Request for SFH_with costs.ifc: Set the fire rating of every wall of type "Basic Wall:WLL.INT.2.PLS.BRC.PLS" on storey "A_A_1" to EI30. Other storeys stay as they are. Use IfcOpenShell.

First a look at what the model holds.

```python
import ifcopenshell
import ifcopenshell.util.element

model = ifcopenshell.open("SFH_with costs.ifc")
print(model.schema)
storey = next(s for s in model.by_type("IfcBuildingStorey") if s.Name == "A_A_1")
walls = [e for e in ifcopenshell.util.element.get_decomposition(storey) if e.is_a("IfcWall")]
seen = {}
for e in walls:
    element_type = ifcopenshell.util.element.get_type(e)
    key = (element_type.Name if element_type != e and element_type else None, ifcopenshell.util.element.get_pset(e, "Pset_WallCommon", "FireRating"))
    seen[key] = seen.get(key, 0) + 1
for (name, value), count in sorted(seen.items(), key=str):
    print(count, "x", name, "|", value)
```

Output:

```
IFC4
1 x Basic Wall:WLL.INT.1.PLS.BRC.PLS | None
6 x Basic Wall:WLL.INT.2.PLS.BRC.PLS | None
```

```python
import ifcopenshell
import ifcopenshell.api.pset
import ifcopenshell.util.element

model = ifcopenshell.open("SFH_with costs.ifc")

storey = next(s for s in model.by_type("IfcBuildingStorey") if s.Name == "A_A_1")
walls = [e for e in ifcopenshell.util.element.get_decomposition(storey) if e.is_a("IfcWall")]

count = 0
for e in walls:
    element_type = ifcopenshell.util.element.get_type(e)
    if element_type in (None, e) or element_type.Name != "Basic Wall:WLL.INT.2.PLS.BRC.PLS":
        continue
    # add_pset returns the element's existing set when there is one.
    pset = ifcopenshell.api.pset.add_pset(model, product=e, name="Pset_WallCommon")
    ifcopenshell.api.pset.edit_pset(model, pset=pset, properties={"FireRating": "EI30"})
    count += 1

print(count, "walls updated")

model.write("SFH_with costs_rev.ifc")
```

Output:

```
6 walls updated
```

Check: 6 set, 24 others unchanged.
